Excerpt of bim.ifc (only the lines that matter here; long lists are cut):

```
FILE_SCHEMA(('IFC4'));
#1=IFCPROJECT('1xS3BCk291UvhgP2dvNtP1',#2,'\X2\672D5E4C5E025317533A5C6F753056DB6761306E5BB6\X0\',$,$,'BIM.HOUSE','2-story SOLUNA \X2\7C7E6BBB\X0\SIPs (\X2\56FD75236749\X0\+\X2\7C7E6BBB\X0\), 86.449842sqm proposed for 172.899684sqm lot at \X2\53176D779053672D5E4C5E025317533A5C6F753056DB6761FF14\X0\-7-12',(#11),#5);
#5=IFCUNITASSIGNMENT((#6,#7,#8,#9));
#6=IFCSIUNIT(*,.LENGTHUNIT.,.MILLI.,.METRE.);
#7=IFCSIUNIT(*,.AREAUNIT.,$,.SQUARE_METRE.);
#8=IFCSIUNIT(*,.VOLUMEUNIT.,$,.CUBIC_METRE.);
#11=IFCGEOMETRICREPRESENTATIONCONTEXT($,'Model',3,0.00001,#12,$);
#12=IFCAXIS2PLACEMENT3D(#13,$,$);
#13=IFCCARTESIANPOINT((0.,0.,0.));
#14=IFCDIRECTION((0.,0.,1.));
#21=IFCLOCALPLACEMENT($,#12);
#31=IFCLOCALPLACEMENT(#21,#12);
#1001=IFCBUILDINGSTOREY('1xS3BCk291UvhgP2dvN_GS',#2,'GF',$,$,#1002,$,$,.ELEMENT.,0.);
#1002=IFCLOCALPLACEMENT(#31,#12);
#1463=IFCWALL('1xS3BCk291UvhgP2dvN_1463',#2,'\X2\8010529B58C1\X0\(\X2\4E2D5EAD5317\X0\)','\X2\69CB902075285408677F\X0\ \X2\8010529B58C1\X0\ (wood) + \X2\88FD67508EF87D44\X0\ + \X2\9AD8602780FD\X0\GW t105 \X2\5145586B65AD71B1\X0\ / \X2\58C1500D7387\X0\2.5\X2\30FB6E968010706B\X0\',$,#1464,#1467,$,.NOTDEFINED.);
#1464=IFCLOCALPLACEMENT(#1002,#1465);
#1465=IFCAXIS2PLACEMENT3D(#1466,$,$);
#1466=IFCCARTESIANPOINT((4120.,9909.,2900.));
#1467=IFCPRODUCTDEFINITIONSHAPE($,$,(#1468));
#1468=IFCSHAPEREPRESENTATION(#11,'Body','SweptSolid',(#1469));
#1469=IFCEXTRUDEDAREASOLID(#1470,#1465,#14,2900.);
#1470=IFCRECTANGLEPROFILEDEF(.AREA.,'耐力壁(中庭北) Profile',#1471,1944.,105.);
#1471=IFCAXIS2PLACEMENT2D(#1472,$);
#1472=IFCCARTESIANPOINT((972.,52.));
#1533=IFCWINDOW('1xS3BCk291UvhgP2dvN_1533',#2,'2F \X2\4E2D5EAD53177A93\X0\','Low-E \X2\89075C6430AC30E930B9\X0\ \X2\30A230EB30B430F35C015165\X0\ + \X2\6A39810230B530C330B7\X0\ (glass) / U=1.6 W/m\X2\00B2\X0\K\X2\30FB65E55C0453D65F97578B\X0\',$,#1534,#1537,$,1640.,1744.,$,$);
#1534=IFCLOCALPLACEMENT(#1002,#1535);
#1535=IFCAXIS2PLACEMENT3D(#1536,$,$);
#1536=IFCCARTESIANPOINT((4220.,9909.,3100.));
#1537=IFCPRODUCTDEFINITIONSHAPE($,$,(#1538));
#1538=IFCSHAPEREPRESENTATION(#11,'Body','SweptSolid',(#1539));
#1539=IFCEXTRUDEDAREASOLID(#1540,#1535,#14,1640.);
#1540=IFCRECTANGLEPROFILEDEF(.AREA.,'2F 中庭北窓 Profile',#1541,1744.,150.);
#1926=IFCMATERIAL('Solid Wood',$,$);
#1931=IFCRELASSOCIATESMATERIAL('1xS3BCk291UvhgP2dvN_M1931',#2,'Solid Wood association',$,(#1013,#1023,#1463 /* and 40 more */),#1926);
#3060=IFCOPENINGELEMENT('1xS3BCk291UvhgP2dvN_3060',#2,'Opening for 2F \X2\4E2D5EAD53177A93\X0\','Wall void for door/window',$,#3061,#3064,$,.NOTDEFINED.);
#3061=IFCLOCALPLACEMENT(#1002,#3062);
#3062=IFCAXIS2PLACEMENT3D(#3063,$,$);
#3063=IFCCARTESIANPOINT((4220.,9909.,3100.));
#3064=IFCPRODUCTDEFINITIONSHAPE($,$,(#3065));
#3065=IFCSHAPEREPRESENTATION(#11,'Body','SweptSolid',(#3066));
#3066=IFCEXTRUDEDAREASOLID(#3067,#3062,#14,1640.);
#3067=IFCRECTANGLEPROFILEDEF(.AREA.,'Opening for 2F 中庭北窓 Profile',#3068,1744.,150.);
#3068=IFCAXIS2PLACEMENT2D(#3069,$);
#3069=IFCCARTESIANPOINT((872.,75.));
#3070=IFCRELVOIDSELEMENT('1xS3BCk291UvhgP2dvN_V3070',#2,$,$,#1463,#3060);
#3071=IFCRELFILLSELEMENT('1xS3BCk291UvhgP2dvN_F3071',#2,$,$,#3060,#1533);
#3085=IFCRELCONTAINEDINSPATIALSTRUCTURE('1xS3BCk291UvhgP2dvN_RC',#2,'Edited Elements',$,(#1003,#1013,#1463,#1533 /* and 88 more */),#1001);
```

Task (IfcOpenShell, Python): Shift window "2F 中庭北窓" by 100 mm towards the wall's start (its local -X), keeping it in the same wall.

```python
import ifcopenshell
import ifcopenshell.api.geometry
import ifcopenshell.util.placement
import ifcopenshell.util.unit

model = ifcopenshell.open("bim.ifc")
unit_scale = ifcopenshell.util.unit.calculate_unit_scale(model)

window = model.by_guid("1xS3BCk291UvhgP2dvN_1533")
opening = window.FillsVoids[0].RelatingOpeningElement
wall = opening.VoidsElements[0].RelatingBuildingElement

wall_matrix = ifcopenshell.util.placement.get_local_placement(wall.ObjectPlacement)
shift = wall_matrix[:3, 0] * -0.1 / unit_scale
before = ifcopenshell.util.placement.get_local_placement(window.ObjectPlacement)[:3, 3].copy()

# The window is not placed relative to its opening, so move both.
for product in (opening, window):
    matrix = ifcopenshell.util.placement.get_local_placement(product.ObjectPlacement)
    matrix[:3, 3] += shift
    ifcopenshell.api.geometry.edit_object_placement(model, product=product, matrix=matrix, is_si=False)

after = ifcopenshell.util.placement.get_local_placement(window.ObjectPlacement)[:3, 3]
print("window moved by", (after - before).round(3) + 0.0)

model.write("bim_updated.ifc")
```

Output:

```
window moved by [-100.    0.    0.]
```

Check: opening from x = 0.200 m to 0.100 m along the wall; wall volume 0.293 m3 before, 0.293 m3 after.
